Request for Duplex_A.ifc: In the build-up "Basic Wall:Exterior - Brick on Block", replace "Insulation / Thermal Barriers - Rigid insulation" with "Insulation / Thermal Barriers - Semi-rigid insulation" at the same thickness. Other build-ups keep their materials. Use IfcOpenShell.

First a look at what the model holds.

```python
import ifcopenshell
import ifcopenshell.util.element

model = ifcopenshell.open("Duplex_A.ifc")
print(model.schema)
for layer_set in model.by_type("IfcMaterialLayerSet"):
    if layer_set.LayerSetName == "Basic Wall:Exterior - Brick on Block":
        for layer in layer_set.MaterialLayers:
            print(layer.id(), layer.Material and layer.Material.Name, layer.LayerThickness, sep=" | ")
        print(len(ifcopenshell.util.element.get_elements_by_material(model, layer_set)), "elements and types use it")
print(sorted(m.Name for m in model.by_type("IfcMaterial") if m.Name)[:60])
```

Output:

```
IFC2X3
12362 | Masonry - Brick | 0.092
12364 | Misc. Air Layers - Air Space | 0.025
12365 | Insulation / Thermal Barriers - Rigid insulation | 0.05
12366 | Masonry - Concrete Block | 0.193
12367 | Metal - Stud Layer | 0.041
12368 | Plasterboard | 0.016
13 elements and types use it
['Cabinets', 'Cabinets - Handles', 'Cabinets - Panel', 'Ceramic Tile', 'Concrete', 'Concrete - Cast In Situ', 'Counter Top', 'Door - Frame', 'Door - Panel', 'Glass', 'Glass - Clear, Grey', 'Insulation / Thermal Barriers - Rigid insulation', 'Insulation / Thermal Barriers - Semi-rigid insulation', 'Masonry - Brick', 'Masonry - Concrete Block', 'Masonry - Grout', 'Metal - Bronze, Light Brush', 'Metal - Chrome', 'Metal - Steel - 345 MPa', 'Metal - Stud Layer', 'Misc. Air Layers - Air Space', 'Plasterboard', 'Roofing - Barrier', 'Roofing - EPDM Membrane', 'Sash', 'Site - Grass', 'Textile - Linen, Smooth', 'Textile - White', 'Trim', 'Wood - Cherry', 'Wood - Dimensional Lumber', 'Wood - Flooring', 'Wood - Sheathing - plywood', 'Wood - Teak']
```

```python
import ifcopenshell
import ifcopenshell.api.material

model = ifcopenshell.open("Duplex_A.ifc")

layer_set = next(s for s in model.by_type("IfcMaterialLayerSet") if s.LayerSetName == "Basic Wall:Exterior - Brick on Block")
layer = next(l for l in layer_set.MaterialLayers if l.Material and l.Material.Name == "Insulation / Thermal Barriers - Rigid insulation")
material = next(m for m in model.by_type("IfcMaterial") if m.Name == "Insulation / Thermal Barriers - Semi-rigid insulation")

# Point this one layer at the other material; renaming the old one would change it everywhere.
ifcopenshell.api.material.edit_layer(model, layer=layer, attributes={}, material=material)

print([l.Material.Name if l.Material else None for l in layer_set.MaterialLayers])

model.write("Duplex_A-out.ifc")
```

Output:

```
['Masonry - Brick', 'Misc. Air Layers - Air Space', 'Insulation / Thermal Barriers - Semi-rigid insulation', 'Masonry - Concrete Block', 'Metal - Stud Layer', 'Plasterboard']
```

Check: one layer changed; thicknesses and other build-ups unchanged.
